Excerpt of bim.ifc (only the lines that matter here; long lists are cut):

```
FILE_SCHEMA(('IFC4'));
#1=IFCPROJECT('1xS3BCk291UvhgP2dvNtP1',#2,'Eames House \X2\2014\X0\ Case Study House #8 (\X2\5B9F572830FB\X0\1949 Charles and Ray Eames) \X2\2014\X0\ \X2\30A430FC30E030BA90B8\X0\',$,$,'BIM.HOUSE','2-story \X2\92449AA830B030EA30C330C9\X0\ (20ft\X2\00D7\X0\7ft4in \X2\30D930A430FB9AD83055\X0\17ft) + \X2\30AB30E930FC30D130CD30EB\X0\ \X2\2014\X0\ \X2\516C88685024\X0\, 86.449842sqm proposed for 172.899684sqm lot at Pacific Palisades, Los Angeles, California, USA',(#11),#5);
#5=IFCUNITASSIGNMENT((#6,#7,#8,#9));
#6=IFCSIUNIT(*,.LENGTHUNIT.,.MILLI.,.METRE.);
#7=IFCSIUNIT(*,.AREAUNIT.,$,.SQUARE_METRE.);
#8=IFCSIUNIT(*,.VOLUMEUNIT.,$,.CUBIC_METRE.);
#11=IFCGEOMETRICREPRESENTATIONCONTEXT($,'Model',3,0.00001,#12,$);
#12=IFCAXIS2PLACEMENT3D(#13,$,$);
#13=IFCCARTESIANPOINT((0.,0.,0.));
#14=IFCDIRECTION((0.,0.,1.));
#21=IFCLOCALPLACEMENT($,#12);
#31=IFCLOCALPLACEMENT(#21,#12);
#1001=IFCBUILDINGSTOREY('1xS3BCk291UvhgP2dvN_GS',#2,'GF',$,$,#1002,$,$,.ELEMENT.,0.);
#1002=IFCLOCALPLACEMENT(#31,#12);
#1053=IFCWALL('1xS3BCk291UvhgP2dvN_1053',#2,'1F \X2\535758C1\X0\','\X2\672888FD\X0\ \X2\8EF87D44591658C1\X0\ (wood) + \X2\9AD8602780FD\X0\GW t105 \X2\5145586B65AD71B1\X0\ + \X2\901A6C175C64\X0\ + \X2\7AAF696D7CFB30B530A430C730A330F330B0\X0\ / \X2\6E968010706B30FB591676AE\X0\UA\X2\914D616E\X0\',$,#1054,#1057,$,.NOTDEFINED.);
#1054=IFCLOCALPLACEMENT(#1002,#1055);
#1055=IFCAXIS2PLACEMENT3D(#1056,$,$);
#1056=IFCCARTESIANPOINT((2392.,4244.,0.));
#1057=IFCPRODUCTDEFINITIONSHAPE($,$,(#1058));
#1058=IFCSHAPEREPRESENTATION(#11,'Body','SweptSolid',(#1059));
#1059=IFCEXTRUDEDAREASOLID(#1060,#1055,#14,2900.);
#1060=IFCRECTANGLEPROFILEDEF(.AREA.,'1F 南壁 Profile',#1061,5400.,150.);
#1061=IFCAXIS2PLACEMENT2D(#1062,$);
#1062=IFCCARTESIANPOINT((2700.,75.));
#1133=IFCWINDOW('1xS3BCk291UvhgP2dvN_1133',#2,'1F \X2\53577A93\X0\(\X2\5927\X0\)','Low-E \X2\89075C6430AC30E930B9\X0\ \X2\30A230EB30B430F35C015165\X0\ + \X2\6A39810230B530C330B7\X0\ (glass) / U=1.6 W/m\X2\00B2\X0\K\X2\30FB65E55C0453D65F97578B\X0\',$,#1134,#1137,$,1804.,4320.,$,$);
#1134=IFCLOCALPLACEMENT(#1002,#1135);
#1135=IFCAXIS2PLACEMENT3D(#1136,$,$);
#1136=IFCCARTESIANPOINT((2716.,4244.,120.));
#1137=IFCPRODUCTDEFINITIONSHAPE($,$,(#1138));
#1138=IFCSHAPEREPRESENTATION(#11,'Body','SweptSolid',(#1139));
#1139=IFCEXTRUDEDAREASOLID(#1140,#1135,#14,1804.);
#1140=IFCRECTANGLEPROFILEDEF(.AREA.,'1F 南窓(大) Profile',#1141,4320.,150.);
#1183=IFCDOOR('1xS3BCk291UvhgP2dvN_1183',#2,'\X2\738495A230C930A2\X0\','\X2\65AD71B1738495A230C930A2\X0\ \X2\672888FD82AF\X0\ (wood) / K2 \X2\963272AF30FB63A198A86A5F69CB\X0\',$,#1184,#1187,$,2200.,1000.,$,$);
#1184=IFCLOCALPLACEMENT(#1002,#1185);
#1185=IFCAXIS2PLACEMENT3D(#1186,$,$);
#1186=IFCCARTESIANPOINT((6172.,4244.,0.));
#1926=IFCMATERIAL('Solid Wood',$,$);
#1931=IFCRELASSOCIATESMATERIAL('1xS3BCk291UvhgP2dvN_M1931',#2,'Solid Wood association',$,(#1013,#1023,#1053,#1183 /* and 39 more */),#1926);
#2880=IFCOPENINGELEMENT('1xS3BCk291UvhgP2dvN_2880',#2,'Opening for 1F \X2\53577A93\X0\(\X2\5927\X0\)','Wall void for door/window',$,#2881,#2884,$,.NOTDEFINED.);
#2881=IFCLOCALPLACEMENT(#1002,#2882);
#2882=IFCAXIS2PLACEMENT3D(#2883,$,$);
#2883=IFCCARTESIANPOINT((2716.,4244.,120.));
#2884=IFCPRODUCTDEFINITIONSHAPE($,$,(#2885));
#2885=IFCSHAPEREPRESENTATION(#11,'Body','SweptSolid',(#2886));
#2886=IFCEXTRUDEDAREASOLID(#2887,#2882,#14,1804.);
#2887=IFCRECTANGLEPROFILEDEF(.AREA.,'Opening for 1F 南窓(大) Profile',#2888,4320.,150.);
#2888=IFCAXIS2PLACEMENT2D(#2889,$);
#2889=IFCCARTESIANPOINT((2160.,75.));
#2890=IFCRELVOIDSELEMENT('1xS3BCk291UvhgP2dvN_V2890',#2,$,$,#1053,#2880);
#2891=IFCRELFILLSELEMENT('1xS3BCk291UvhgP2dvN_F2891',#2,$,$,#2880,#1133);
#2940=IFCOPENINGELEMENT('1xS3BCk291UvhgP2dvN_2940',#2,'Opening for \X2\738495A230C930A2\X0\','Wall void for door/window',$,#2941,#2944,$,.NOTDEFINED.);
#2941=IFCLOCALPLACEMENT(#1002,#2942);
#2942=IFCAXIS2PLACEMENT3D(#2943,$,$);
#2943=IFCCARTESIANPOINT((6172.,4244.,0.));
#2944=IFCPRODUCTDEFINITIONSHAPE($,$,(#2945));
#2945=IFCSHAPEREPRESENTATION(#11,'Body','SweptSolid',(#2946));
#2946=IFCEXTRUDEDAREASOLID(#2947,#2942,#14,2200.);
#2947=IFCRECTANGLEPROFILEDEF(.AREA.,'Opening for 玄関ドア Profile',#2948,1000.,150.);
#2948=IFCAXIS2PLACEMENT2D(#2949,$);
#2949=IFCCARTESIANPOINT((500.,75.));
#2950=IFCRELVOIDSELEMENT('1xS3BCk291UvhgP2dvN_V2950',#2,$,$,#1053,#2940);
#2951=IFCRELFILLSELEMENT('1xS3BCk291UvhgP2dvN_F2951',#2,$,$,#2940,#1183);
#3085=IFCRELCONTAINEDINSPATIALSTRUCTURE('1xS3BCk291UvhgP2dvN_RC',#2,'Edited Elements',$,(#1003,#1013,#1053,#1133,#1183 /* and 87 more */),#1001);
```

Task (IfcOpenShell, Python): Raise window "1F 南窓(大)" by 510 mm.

```python
import numpy as np
import ifcopenshell
import ifcopenshell.api.geometry
import ifcopenshell.util.placement
import ifcopenshell.util.unit

model = ifcopenshell.open("bim.ifc")
unit_scale = ifcopenshell.util.unit.calculate_unit_scale(model)

window = model.by_guid("1xS3BCk291UvhgP2dvN_1133")
opening = window.FillsVoids[0].RelatingOpeningElement
dz = 0.51 / unit_scale

shift = np.array([0.0, 0.0, dz])
# The window is not placed relative to its opening, so move both.
for product in (opening, window):
    matrix = ifcopenshell.util.placement.get_local_placement(product.ObjectPlacement)
    matrix[:3, 3] += shift
    ifcopenshell.api.geometry.edit_object_placement(model, product=product, matrix=matrix, is_si=False)

print(f"moved by {dz * unit_scale:+.3f} m")

model.write("bim_v2.ifc")
```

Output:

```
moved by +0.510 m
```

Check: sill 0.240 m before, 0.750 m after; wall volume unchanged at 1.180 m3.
